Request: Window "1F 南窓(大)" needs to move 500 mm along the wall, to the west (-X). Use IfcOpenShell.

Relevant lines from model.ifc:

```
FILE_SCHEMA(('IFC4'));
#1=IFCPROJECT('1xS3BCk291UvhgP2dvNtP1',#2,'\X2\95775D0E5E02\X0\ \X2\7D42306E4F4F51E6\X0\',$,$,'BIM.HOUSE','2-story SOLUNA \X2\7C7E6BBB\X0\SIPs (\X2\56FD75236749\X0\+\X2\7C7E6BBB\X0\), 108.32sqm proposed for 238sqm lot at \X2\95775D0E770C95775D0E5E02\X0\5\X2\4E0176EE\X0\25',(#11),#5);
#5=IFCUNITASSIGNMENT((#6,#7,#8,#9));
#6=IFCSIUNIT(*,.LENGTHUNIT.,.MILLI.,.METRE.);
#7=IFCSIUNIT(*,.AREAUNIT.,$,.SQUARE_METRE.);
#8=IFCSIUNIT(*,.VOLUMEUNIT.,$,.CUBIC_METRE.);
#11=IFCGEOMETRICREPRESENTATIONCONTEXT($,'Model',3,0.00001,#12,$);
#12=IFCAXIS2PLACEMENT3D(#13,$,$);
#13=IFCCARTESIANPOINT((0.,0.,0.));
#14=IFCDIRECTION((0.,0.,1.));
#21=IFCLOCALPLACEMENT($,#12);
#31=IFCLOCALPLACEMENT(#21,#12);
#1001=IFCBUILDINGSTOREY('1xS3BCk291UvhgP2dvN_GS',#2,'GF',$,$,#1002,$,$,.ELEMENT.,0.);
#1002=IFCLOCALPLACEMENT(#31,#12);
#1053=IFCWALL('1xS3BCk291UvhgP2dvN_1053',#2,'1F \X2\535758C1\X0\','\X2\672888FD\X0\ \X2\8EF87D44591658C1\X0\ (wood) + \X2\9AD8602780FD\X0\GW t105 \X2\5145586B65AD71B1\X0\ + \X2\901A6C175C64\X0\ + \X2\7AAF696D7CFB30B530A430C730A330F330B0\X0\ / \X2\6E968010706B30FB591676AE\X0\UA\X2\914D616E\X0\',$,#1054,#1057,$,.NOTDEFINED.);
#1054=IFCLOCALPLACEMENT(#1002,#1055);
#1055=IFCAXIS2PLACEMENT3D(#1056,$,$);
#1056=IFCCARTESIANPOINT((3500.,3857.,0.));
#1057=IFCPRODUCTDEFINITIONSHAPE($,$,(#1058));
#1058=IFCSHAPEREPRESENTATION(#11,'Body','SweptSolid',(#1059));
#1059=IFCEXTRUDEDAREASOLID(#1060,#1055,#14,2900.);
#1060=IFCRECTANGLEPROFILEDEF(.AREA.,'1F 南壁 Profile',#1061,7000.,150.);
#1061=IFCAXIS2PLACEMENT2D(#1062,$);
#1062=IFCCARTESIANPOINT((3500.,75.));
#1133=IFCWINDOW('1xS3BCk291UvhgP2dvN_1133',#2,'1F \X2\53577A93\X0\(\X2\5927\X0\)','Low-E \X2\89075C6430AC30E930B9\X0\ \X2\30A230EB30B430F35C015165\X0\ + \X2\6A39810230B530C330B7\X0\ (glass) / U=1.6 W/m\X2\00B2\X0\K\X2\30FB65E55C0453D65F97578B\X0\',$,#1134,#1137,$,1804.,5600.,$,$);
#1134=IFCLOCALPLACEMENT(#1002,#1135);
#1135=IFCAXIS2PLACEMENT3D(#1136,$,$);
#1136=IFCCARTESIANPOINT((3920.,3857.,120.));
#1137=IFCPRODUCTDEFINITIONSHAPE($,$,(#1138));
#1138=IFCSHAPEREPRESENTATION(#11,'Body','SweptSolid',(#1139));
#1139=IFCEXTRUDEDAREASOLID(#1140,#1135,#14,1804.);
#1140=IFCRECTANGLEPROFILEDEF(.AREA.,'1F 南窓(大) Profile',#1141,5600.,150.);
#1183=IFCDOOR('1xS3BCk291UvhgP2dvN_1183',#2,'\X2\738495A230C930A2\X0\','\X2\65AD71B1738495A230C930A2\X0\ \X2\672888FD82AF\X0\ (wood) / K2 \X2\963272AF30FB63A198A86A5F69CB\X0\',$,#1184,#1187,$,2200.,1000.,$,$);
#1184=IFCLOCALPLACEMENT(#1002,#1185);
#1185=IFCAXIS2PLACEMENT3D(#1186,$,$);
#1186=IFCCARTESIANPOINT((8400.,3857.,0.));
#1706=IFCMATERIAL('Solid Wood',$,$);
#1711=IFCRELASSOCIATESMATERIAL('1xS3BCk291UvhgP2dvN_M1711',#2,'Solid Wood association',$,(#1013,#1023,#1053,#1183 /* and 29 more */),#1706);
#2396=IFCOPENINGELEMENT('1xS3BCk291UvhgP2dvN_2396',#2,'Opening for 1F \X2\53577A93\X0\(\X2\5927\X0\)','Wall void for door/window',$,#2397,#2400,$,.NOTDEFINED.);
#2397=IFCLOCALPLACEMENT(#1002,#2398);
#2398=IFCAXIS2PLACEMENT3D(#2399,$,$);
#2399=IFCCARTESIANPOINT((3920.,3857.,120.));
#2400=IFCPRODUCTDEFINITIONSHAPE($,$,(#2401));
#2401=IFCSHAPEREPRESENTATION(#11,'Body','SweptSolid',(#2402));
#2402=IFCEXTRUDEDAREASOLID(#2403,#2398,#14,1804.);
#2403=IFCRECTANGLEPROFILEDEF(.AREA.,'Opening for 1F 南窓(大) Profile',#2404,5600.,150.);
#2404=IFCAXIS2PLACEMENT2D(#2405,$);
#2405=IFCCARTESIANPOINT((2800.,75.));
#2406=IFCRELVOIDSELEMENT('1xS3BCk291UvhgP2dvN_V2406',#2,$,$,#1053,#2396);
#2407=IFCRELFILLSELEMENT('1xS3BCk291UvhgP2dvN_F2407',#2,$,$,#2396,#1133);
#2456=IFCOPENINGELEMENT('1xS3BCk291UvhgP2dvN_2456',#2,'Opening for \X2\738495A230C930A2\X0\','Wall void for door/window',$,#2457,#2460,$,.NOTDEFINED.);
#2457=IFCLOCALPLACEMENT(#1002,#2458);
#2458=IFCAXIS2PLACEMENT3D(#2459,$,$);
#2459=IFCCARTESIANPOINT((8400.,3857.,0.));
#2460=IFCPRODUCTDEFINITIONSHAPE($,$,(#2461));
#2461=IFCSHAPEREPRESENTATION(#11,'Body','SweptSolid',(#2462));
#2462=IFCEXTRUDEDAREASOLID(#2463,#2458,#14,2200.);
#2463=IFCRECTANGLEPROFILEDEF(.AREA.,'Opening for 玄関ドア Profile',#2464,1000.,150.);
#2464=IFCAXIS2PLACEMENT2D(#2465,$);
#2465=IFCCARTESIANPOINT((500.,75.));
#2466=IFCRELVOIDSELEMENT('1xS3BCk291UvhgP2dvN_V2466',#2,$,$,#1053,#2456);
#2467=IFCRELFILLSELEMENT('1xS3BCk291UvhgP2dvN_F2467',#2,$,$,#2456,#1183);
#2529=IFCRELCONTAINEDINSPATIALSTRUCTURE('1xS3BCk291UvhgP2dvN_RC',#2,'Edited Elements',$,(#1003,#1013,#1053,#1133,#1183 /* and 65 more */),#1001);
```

```python
import ifcopenshell
import ifcopenshell.api.geometry
import ifcopenshell.util.placement

model = ifcopenshell.open("model.ifc")

window = model.by_guid("1xS3BCk291UvhgP2dvN_1133")
opening = window.FillsVoids[0].RelatingOpeningElement
wall = opening.VoidsElements[0].RelatingBuildingElement

wall_matrix = ifcopenshell.util.placement.get_local_placement(wall.ObjectPlacement)
shift = wall_matrix[:3, 0] * -500.0
before = ifcopenshell.util.placement.get_local_placement(window.ObjectPlacement)[:3, 3].copy()

# The window is not placed relative to its opening, so move both.
for product in (opening, window):
    matrix = ifcopenshell.util.placement.get_local_placement(product.ObjectPlacement)
    matrix[:3, 3] += shift
    ifcopenshell.api.geometry.edit_object_placement(model, product=product, matrix=matrix, is_si=False)

after = ifcopenshell.util.placement.get_local_placement(window.ObjectPlacement)[:3, 3]
print("window moved by", (after - before).round(3) + 0.0)

model.write("model_v2.ifc")
```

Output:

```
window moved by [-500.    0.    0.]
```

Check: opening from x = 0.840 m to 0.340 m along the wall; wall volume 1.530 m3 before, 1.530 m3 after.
